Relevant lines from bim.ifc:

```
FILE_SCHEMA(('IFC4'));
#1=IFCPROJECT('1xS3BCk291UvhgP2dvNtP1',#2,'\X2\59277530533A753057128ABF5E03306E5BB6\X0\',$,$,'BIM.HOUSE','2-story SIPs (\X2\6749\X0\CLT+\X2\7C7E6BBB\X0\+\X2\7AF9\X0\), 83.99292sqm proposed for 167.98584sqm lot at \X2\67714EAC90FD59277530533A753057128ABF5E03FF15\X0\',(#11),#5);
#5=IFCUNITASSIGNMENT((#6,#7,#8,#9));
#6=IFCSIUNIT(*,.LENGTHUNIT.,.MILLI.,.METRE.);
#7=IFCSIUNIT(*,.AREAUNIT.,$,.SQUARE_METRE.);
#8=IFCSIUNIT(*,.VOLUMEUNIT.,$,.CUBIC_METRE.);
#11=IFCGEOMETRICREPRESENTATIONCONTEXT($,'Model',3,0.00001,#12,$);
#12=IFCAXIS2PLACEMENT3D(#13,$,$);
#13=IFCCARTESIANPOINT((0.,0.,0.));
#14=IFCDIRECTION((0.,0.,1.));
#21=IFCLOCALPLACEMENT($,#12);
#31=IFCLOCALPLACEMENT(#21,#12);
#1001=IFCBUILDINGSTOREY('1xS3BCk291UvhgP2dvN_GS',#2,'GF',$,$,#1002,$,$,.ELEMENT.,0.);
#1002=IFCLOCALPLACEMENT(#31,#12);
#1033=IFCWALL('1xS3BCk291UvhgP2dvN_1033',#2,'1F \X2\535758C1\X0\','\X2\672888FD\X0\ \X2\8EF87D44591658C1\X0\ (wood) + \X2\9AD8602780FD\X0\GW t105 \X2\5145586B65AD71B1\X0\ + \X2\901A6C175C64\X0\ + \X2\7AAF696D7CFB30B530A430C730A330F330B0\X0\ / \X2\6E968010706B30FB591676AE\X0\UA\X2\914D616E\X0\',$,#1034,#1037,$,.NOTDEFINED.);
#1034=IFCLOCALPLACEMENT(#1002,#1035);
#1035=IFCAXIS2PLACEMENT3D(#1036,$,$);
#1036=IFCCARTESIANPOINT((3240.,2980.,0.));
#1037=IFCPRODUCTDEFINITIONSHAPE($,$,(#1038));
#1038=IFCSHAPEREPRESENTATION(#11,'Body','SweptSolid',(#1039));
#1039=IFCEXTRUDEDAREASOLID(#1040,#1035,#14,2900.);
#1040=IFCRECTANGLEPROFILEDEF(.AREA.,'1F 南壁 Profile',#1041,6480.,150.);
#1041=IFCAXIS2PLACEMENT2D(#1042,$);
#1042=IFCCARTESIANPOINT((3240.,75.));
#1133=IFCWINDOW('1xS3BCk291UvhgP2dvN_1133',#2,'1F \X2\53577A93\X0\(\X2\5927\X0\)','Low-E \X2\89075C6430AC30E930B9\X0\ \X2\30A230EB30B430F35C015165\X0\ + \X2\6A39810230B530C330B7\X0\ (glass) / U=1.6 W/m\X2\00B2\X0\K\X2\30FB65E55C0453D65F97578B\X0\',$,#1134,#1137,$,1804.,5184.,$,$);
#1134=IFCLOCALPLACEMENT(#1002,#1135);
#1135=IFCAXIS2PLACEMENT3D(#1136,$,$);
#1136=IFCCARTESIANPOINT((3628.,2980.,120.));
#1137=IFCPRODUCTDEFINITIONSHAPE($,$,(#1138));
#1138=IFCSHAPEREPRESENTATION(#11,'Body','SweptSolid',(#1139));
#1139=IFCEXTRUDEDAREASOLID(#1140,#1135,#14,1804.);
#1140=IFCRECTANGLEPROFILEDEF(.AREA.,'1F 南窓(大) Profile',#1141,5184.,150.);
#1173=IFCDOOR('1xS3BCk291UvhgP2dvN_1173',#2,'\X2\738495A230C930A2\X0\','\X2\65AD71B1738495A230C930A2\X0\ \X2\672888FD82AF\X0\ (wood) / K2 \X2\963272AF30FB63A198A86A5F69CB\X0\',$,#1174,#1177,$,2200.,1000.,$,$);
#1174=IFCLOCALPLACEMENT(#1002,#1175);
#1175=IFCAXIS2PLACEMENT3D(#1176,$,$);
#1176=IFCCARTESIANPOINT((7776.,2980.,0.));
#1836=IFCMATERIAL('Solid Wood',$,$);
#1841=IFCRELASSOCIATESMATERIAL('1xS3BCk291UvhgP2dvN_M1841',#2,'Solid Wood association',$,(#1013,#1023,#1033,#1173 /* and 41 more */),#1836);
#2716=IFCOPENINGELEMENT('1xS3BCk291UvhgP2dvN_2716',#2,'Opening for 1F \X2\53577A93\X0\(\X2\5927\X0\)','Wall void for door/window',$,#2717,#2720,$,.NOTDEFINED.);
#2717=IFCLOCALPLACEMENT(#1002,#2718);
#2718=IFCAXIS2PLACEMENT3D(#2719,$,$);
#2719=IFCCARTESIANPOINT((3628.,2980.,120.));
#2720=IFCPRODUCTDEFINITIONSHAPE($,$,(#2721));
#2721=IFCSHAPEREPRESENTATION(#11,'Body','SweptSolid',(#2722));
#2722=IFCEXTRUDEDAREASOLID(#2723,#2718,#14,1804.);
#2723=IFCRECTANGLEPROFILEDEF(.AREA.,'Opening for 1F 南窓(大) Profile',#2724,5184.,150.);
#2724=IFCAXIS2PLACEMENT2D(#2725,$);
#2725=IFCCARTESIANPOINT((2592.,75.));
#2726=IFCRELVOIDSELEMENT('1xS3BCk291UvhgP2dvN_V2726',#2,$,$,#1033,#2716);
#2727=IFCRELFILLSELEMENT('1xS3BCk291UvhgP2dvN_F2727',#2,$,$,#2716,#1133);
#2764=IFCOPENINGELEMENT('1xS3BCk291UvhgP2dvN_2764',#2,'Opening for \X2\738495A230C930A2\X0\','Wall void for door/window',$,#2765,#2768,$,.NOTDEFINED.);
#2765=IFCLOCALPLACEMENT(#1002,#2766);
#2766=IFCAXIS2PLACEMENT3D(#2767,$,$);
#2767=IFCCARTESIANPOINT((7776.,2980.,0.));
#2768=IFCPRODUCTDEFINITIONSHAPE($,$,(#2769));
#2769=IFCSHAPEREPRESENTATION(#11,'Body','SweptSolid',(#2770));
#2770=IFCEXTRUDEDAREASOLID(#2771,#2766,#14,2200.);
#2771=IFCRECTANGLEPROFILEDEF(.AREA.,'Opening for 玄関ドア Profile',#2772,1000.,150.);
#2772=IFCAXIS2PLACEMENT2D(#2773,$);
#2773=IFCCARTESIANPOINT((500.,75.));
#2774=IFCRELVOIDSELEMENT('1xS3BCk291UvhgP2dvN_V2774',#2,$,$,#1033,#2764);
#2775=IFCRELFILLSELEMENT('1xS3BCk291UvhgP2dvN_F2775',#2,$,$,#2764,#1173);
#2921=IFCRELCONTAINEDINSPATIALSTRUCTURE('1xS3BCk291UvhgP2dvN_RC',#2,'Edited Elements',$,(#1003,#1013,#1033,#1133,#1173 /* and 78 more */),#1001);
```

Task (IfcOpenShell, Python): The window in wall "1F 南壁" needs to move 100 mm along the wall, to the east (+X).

```python
import ifcopenshell
import ifcopenshell.api.geometry
import ifcopenshell.util.placement
import ifcopenshell.util.unit

model = ifcopenshell.open("bim.ifc")
unit_scale = ifcopenshell.util.unit.calculate_unit_scale(model)

window = model.by_guid("1xS3BCk291UvhgP2dvN_1133")
opening = window.FillsVoids[0].RelatingOpeningElement
wall = opening.VoidsElements[0].RelatingBuildingElement

wall_matrix = ifcopenshell.util.placement.get_local_placement(wall.ObjectPlacement)
shift = wall_matrix[:3, 0] * 0.1 / unit_scale
before = ifcopenshell.util.placement.get_local_placement(window.ObjectPlacement)[:3, 3].copy()

# The window is not placed relative to its opening, so move both.
for product in (opening, window):
    matrix = ifcopenshell.util.placement.get_local_placement(product.ObjectPlacement)
    matrix[:3, 3] += shift
    ifcopenshell.api.geometry.edit_object_placement(model, product=product, matrix=matrix, is_si=False)

after = ifcopenshell.util.placement.get_local_placement(window.ObjectPlacement)[:3, 3]
print("window moved by", (after - before).round(3) + 0.0)

model.write("bim-out.ifc")
```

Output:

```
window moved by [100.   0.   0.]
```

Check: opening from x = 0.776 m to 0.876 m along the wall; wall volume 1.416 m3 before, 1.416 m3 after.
